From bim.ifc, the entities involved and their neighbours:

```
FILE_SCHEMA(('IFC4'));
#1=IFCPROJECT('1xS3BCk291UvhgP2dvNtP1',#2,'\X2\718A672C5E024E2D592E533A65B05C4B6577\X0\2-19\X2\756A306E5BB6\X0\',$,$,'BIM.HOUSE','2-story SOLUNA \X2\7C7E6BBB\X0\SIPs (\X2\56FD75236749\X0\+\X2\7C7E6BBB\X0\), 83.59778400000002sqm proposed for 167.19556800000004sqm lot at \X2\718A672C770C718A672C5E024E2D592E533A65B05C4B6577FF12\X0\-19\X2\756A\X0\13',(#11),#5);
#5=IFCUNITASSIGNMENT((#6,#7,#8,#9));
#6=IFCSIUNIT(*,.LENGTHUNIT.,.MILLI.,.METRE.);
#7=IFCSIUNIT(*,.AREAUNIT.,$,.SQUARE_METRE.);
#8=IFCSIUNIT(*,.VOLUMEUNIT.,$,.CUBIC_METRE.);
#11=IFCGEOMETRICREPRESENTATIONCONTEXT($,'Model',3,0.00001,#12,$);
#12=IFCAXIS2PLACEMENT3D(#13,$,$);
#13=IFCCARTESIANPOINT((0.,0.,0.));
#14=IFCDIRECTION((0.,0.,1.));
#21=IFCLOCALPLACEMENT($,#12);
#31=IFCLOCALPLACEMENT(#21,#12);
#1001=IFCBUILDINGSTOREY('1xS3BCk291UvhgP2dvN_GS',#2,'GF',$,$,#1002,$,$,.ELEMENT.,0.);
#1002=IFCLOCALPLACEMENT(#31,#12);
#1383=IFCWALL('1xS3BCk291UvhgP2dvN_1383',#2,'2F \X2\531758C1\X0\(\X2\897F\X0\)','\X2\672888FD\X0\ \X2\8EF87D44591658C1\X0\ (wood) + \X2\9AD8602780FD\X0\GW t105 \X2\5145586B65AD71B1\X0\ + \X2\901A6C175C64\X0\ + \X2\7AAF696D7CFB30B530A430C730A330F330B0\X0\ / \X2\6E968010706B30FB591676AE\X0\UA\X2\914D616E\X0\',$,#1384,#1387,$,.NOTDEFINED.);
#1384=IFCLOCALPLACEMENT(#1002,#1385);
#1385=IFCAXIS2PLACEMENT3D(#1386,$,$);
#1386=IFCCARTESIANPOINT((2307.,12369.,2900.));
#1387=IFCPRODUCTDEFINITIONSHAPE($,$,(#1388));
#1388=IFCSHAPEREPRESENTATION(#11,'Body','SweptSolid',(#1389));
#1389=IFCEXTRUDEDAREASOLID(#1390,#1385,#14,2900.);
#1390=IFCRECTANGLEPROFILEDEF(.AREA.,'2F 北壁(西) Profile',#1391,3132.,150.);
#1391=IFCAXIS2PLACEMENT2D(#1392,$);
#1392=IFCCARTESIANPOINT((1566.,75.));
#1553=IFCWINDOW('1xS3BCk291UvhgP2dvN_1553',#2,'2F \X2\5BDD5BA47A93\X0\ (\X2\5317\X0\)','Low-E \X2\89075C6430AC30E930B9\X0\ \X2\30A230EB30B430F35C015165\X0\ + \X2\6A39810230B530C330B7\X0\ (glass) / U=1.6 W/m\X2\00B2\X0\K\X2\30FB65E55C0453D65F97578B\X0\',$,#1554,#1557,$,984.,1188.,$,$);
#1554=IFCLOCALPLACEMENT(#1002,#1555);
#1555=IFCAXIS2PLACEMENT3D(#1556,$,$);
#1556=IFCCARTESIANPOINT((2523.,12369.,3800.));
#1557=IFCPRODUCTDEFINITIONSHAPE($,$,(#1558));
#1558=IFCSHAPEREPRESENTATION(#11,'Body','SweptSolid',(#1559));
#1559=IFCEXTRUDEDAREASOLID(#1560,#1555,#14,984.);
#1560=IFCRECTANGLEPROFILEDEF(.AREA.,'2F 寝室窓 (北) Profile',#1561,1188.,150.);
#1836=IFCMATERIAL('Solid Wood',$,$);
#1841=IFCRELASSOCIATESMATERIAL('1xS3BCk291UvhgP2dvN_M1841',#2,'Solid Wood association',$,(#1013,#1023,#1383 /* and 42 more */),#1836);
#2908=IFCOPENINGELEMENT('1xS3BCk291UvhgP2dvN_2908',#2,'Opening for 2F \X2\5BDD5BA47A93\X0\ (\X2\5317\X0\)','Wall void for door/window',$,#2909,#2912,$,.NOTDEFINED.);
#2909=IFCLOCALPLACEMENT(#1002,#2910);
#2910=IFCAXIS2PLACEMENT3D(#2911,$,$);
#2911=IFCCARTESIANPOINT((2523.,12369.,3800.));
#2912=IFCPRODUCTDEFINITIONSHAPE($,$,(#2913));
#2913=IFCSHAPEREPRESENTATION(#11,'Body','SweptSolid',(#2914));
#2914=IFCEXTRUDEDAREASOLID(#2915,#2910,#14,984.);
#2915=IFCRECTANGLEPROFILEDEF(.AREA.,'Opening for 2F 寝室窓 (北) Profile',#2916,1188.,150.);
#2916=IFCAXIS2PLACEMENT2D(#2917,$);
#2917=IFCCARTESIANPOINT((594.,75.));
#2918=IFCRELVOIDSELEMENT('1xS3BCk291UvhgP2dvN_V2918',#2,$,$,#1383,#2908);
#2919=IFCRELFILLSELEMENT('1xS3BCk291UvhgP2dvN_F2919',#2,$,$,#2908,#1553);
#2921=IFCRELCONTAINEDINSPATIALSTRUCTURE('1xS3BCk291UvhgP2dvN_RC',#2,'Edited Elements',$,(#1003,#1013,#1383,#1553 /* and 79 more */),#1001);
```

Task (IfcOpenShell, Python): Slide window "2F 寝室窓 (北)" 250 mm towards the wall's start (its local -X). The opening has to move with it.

```python
import ifcopenshell
import ifcopenshell.api.geometry
import ifcopenshell.util.placement
import ifcopenshell.util.unit

model = ifcopenshell.open("bim.ifc")
unit_scale = ifcopenshell.util.unit.calculate_unit_scale(model)

window = model.by_guid("1xS3BCk291UvhgP2dvN_1553")
opening = window.FillsVoids[0].RelatingOpeningElement
wall = opening.VoidsElements[0].RelatingBuildingElement

wall_matrix = ifcopenshell.util.placement.get_local_placement(wall.ObjectPlacement)
shift = wall_matrix[:3, 0] * -0.25 / unit_scale
before = ifcopenshell.util.placement.get_local_placement(window.ObjectPlacement)[:3, 3].copy()

# The window is not placed relative to its opening, so move both.
for product in (opening, window):
    matrix = ifcopenshell.util.placement.get_local_placement(product.ObjectPlacement)
    matrix[:3, 3] += shift
    ifcopenshell.api.geometry.edit_object_placement(model, product=product, matrix=matrix, is_si=False)

after = ifcopenshell.util.placement.get_local_placement(window.ObjectPlacement)[:3, 3]
print("window moved by", (after - before).round(3) + 0.0)

model.write("bim_rev.ifc")
```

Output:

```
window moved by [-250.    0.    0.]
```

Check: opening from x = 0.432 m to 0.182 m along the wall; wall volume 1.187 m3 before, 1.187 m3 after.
